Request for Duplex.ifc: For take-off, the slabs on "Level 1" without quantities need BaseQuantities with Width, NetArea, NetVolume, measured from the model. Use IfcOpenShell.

First a look at what the model holds.

```python
import ifcopenshell
import ifcopenshell.util.element
import ifcopenshell.util.unit

model = ifcopenshell.open("Duplex.ifc")
print(model.schema)
for unit_type in ("LENGTHUNIT", "AREAUNIT", "VOLUMEUNIT"):
    print(unit_type, ifcopenshell.util.unit.calculate_unit_scale(model, unit_type))
storey = next(s for s in model.by_type("IfcBuildingStorey") if s.Name == "Level 1")
slabs = [e for e in ifcopenshell.util.element.get_decomposition(storey) if e.is_a("IfcSlab")]
for e in sorted(slabs, key=lambda e: e.id()):
    print(e.id(), e.is_a(), e.Name, list(ifcopenshell.util.element.get_psets(e, qtos_only=True)), sep=" | ")
```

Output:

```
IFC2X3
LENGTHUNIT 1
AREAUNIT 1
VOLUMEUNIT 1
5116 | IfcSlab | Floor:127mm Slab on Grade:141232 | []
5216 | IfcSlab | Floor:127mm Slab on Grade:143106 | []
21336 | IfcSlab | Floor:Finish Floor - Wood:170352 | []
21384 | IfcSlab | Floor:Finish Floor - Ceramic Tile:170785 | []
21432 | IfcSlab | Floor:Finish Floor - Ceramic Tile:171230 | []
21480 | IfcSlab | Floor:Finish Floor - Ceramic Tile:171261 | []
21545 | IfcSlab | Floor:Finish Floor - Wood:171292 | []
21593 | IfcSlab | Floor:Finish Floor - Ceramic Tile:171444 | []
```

```python
import ifcopenshell
import ifcopenshell.api.pset
import ifcopenshell.geom
import ifcopenshell.util.element
import ifcopenshell.util.shape
import ifcopenshell.util.unit

model = ifcopenshell.open("Duplex.ifc")
unit_scale = ifcopenshell.util.unit.calculate_unit_scale(model)
area_scale = ifcopenshell.util.unit.calculate_unit_scale(model, "AREAUNIT")
volume_scale = ifcopenshell.util.unit.calculate_unit_scale(model, "VOLUMEUNIT")
settings = ifcopenshell.geom.settings()

storey = next(s for s in model.by_type("IfcBuildingStorey") if s.Name == "Level 1")
slabs = [e for e in ifcopenshell.util.element.get_decomposition(storey) if e.is_a("IfcSlab")]

for e in sorted(slabs, key=lambda e: e.id()):
    if ifcopenshell.util.element.get_psets(e, qtos_only=True, should_inherit=False):
        continue
    # Geometry comes back in metres, in the element's own axes.
    shape = ifcopenshell.geom.create_shape(settings, e)
    values = {
        "Width": ifcopenshell.util.shape.get_z(shape.geometry) / unit_scale,
        "NetArea": ifcopenshell.util.shape.get_footprint_area(shape.geometry) / area_scale,
        "NetVolume": ifcopenshell.util.shape.get_volume(shape.geometry) / volume_scale,
    }
    qto = ifcopenshell.api.pset.add_qto(model, product=e, name="BaseQuantities")
    ifcopenshell.api.pset.edit_qto(model, qto=qto, properties=values)
    print(e.id(), {k: round(v, 3) for k, v in values.items()})

model.write("Duplex_edited.ifc")
```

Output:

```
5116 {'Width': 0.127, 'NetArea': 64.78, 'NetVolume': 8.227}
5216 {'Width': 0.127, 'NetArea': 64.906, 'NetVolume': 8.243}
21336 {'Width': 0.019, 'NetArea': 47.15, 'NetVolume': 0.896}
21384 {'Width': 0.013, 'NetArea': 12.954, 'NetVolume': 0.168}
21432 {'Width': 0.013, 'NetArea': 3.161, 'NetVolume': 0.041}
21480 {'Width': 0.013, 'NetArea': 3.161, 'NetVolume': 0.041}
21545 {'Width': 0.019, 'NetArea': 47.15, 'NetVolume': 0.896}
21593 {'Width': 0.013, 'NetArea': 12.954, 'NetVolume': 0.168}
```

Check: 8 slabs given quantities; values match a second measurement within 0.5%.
